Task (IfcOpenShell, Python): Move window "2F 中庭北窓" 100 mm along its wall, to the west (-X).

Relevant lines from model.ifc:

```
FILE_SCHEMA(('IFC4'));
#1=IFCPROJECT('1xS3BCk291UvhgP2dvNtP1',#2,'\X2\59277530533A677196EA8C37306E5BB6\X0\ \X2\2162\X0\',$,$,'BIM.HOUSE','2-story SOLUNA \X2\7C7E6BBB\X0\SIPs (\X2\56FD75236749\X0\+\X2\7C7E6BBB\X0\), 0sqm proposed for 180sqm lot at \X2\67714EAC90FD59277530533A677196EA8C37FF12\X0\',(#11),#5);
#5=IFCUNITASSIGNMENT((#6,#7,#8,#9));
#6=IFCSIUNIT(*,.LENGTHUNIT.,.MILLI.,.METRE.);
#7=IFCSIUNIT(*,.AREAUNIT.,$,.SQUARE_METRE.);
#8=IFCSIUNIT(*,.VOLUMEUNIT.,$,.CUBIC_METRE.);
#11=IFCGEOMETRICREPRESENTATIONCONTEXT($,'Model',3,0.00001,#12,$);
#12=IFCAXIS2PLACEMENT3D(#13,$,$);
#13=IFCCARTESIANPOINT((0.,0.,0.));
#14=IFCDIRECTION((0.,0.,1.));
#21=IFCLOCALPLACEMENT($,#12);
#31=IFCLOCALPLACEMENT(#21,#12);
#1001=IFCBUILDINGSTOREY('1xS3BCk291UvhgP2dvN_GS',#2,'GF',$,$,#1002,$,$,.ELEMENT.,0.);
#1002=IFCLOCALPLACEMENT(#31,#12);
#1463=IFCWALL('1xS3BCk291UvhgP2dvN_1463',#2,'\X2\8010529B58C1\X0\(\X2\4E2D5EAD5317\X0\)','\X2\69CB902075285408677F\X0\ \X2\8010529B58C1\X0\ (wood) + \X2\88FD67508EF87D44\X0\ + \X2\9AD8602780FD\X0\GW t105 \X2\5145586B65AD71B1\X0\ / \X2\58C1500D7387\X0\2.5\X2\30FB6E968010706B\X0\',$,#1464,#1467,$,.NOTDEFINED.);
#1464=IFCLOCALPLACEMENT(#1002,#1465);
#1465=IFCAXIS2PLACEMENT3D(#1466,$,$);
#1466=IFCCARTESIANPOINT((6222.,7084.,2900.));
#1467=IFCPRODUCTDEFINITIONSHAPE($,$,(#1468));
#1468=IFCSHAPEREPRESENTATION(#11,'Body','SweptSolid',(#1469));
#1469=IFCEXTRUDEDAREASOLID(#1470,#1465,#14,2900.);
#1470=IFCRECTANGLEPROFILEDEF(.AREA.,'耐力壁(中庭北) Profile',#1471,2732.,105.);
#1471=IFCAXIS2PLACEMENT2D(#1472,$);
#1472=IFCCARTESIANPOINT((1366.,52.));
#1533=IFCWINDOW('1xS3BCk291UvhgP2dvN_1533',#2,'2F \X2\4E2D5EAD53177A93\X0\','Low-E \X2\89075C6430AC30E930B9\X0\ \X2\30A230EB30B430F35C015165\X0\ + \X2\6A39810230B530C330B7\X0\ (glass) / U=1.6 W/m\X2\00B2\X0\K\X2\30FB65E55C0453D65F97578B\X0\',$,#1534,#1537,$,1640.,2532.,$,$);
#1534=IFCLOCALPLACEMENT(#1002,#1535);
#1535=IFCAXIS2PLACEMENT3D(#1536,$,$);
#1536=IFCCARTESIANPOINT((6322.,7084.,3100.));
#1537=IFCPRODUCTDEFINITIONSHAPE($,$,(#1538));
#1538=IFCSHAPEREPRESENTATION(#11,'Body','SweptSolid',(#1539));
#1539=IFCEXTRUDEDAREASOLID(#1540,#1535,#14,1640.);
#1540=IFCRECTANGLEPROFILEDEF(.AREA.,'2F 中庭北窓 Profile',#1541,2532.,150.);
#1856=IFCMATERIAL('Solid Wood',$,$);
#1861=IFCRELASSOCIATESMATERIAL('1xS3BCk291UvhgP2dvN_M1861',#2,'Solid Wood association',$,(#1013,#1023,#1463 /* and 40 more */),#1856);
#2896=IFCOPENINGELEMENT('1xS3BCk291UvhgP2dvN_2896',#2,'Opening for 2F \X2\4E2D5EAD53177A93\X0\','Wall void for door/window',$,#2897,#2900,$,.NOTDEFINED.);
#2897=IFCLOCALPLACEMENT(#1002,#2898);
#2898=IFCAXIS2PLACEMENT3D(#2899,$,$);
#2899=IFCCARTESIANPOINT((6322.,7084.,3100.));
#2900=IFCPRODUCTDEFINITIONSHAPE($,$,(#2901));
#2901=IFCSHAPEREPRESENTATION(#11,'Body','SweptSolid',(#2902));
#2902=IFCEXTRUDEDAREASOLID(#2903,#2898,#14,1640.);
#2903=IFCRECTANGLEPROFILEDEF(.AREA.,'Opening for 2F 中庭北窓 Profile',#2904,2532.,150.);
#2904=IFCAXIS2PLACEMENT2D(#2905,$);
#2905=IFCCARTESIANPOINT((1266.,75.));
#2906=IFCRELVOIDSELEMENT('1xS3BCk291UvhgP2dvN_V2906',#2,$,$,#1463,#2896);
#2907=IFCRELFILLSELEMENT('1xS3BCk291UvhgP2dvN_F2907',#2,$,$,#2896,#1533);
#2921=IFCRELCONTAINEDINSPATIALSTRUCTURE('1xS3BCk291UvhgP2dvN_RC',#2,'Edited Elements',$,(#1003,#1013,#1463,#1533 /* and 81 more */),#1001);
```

```python
import ifcopenshell
import ifcopenshell.api.geometry
import ifcopenshell.util.placement
import ifcopenshell.util.unit

model = ifcopenshell.open("model.ifc")
unit_scale = ifcopenshell.util.unit.calculate_unit_scale(model)

window = model.by_guid("1xS3BCk291UvhgP2dvN_1533")
opening = window.FillsVoids[0].RelatingOpeningElement
wall = opening.VoidsElements[0].RelatingBuildingElement

wall_matrix = ifcopenshell.util.placement.get_local_placement(wall.ObjectPlacement)
shift = wall_matrix[:3, 0] * -0.1 / unit_scale
before = ifcopenshell.util.placement.get_local_placement(window.ObjectPlacement)[:3, 3].copy()

# The window is not placed relative to its opening, so move both.
for product in (opening, window):
    matrix = ifcopenshell.util.placement.get_local_placement(product.ObjectPlacement)
    matrix[:3, 3] += shift
    ifcopenshell.api.geometry.edit_object_placement(model, product=product, matrix=matrix, is_si=False)

after = ifcopenshell.util.placement.get_local_placement(window.ObjectPlacement)[:3, 3]
print("window moved by", (after - before).round(3) + 0.0)

model.write("model-out.ifc")
```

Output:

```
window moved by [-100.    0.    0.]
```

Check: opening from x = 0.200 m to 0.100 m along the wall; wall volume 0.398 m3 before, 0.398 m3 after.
